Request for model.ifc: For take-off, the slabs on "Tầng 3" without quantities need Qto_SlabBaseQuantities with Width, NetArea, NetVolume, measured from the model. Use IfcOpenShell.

First a look at what the model holds.

```python
import ifcopenshell
import ifcopenshell.util.element
import ifcopenshell.util.unit

model = ifcopenshell.open("model.ifc")
print(model.schema)
for unit_type in ("LENGTHUNIT", "AREAUNIT", "VOLUMEUNIT"):
    print(unit_type, ifcopenshell.util.unit.calculate_unit_scale(model, unit_type))
storey = next(s for s in model.by_type("IfcBuildingStorey") if s.Name == "Tầng 3")
slabs = [e for e in ifcopenshell.util.element.get_decomposition(storey) if e.is_a("IfcSlab")]
for e in sorted(slabs, key=lambda e: e.id()):
    print(e.id(), e.is_a(), e.Name, list(ifcopenshell.util.element.get_psets(e, qtos_only=True)), sep=" | ")
```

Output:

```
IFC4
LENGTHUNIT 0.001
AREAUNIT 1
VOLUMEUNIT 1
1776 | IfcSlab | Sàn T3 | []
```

```python
import ifcopenshell
import ifcopenshell.api.pset
import ifcopenshell.geom
import ifcopenshell.util.element
import ifcopenshell.util.shape
import ifcopenshell.util.unit

model = ifcopenshell.open("model.ifc")
unit_scale = ifcopenshell.util.unit.calculate_unit_scale(model)
area_scale = ifcopenshell.util.unit.calculate_unit_scale(model, "AREAUNIT")
volume_scale = ifcopenshell.util.unit.calculate_unit_scale(model, "VOLUMEUNIT")
settings = ifcopenshell.geom.settings()

storey = next(s for s in model.by_type("IfcBuildingStorey") if s.Name == "Tầng 3")
slabs = [e for e in ifcopenshell.util.element.get_decomposition(storey) if e.is_a("IfcSlab")]

for e in sorted(slabs, key=lambda e: e.id()):
    if ifcopenshell.util.element.get_psets(e, qtos_only=True, should_inherit=False):
        continue
    # Geometry comes back in metres, in the element's own axes.
    shape = ifcopenshell.geom.create_shape(settings, e)
    values = {
        "Width": ifcopenshell.util.shape.get_z(shape.geometry) / unit_scale,
        "NetArea": ifcopenshell.util.shape.get_footprint_area(shape.geometry) / area_scale,
        "NetVolume": ifcopenshell.util.shape.get_volume(shape.geometry) / volume_scale,
    }
    qto = ifcopenshell.api.pset.add_qto(model, product=e, name="Qto_SlabBaseQuantities")
    ifcopenshell.api.pset.edit_qto(model, qto=qto, properties=values)
    print(e.id(), {k: round(v, 3) for k, v in values.items()})

model.write("model-out.ifc")
```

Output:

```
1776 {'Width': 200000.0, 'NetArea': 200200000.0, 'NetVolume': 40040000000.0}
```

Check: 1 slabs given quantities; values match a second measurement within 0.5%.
